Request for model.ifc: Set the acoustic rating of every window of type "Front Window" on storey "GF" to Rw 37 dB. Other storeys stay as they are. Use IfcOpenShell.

First a look at what the model holds.

```python
import ifcopenshell
import ifcopenshell.util.element

model = ifcopenshell.open("model.ifc")
print(model.schema)
storey = next(s for s in model.by_type("IfcBuildingStorey") if s.Name == "GF")
windows = [e for e in ifcopenshell.util.element.get_decomposition(storey) if e.is_a("IfcWindow")]
seen = {}
for e in windows:
    element_type = ifcopenshell.util.element.get_type(e)
    key = (element_type.Name if element_type != e and element_type else None, ifcopenshell.util.element.get_pset(e, "Pset_WindowCommon", "AcousticRating"))
    seen[key] = seen.get(key, 0) + 1
for (name, value), count in sorted(seen.items(), key=str):
    print(count, "x", name, "|", value)
```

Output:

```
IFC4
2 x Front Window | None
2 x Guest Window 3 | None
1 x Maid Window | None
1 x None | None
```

```python
import ifcopenshell
import ifcopenshell.api.pset
import ifcopenshell.util.element

model = ifcopenshell.open("model.ifc")

storey = next(s for s in model.by_type("IfcBuildingStorey") if s.Name == "GF")
windows = [e for e in ifcopenshell.util.element.get_decomposition(storey) if e.is_a("IfcWindow")]

count = 0
for e in windows:
    element_type = ifcopenshell.util.element.get_type(e)
    if element_type in (None, e) or element_type.Name != "Front Window":
        continue
    # add_pset returns the element's existing set when there is one.
    pset = ifcopenshell.api.pset.add_pset(model, product=e, name="Pset_WindowCommon")
    ifcopenshell.api.pset.edit_pset(model, pset=pset, properties={"AcousticRating": "Rw 37 dB"})
    count += 1

print(count, "windows updated")

model.write("model-out.ifc")
```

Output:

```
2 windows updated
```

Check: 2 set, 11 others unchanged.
